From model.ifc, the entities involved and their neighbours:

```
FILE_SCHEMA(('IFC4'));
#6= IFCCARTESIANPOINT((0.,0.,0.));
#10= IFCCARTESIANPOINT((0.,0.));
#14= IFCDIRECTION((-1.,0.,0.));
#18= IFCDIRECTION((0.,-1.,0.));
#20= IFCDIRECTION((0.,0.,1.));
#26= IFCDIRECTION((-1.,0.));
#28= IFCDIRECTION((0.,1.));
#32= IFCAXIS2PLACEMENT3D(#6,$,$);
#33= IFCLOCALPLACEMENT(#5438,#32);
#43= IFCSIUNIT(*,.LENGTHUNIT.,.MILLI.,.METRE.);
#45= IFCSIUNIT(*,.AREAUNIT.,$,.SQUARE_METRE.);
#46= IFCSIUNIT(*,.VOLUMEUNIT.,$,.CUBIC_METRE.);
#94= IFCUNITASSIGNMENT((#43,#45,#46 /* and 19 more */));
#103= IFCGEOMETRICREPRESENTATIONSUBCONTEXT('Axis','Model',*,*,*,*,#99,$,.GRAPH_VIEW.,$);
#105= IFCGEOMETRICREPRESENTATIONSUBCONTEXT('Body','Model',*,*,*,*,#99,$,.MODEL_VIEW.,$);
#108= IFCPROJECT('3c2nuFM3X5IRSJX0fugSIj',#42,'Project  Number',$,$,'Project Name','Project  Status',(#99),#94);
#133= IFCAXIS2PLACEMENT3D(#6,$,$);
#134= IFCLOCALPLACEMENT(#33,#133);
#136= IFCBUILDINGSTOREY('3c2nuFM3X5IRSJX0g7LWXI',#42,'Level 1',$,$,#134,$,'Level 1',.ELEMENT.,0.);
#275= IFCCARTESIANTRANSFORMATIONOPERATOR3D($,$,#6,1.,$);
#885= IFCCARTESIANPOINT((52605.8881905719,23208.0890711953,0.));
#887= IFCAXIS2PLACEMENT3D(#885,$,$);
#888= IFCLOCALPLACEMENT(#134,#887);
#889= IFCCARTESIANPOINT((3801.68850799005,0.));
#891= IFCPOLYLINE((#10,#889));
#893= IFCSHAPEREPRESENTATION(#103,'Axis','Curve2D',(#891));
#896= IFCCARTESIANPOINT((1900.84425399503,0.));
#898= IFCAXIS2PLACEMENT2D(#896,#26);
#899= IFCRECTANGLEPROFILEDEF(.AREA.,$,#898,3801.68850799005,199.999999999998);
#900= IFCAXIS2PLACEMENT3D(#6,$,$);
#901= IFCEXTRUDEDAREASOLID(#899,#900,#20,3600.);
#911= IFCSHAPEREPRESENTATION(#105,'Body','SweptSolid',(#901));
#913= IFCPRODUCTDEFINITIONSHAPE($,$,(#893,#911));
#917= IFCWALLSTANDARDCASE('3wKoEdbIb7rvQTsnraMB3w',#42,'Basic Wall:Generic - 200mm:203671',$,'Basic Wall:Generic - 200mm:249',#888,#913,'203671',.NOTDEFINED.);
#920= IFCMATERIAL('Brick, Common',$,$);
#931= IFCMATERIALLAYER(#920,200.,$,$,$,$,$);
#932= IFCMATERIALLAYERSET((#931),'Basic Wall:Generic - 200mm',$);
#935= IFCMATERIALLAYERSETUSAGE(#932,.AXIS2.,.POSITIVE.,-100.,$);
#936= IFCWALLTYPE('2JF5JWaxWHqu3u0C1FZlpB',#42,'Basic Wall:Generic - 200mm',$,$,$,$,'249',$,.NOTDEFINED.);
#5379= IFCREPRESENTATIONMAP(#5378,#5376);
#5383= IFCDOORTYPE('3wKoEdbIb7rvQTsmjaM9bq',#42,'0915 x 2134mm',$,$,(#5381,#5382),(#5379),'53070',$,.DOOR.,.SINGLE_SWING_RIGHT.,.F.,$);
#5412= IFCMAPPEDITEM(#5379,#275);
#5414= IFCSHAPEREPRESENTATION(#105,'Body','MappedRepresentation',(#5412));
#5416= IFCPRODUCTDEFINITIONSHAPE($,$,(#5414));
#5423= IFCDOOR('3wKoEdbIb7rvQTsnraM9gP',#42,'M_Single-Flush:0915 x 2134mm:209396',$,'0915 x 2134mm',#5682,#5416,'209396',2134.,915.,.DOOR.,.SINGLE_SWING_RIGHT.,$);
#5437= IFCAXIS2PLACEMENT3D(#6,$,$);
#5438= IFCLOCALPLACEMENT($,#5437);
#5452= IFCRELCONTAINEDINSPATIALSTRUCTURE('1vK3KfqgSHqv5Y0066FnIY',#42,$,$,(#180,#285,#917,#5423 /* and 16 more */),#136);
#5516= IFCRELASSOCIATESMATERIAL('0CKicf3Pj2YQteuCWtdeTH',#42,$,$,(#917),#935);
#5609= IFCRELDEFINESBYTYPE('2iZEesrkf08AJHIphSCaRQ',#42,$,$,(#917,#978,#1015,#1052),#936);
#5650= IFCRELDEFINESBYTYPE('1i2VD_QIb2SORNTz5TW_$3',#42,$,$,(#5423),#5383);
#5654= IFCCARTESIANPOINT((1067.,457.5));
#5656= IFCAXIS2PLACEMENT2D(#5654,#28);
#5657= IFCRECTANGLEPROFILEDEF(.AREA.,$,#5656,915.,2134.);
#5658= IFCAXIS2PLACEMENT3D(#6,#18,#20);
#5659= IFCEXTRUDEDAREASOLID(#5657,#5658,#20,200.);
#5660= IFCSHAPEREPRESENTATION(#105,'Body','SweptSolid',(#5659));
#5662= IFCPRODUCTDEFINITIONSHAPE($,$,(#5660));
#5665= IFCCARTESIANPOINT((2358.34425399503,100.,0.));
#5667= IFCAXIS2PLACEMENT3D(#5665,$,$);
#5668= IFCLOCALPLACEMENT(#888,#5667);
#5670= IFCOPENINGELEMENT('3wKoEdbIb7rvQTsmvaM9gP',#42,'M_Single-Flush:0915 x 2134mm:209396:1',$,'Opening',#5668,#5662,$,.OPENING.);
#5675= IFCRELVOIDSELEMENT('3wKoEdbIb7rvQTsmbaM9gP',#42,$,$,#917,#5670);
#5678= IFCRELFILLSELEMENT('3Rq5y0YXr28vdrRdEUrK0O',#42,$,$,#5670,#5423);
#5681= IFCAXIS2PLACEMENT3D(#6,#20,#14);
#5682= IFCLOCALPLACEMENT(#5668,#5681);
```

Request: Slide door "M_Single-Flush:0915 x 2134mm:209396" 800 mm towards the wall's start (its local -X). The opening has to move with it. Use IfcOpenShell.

```python
import ifcopenshell
import ifcopenshell.api.geometry
import ifcopenshell.util.placement
import ifcopenshell.util.unit

model = ifcopenshell.open("model.ifc")
unit_scale = ifcopenshell.util.unit.calculate_unit_scale(model)

door = model.by_id(5423)
opening = door.FillsVoids[0].RelatingOpeningElement
wall = opening.VoidsElements[0].RelatingBuildingElement

wall_matrix = ifcopenshell.util.placement.get_local_placement(wall.ObjectPlacement)
shift = wall_matrix[:3, 0] * -0.8 / unit_scale
before = ifcopenshell.util.placement.get_local_placement(door.ObjectPlacement)[:3, 3].copy()

# The door is placed relative to its opening, so it follows when the opening moves.
matrix = ifcopenshell.util.placement.get_local_placement(opening.ObjectPlacement)
matrix[:3, 3] += shift
ifcopenshell.api.geometry.edit_object_placement(
    model, product=opening, matrix=matrix, is_si=False, should_transform_children=True
)

after = ifcopenshell.util.placement.get_local_placement(door.ObjectPlacement)[:3, 3]
print("door moved by", (after - before).round(3) + 0.0)

model.write("model_v2.ifc")
```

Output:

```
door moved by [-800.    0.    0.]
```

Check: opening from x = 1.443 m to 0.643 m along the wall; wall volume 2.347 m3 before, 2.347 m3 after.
